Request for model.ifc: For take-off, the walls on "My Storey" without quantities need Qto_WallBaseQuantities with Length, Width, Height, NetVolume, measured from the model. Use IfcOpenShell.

First a look at what the model holds.

```python
import ifcopenshell
import ifcopenshell.util.element
import ifcopenshell.util.unit

model = ifcopenshell.open("model.ifc")
print(model.schema)
for unit_type in ("LENGTHUNIT", "AREAUNIT", "VOLUMEUNIT"):
    print(unit_type, ifcopenshell.util.unit.calculate_unit_scale(model, unit_type))
storey = next(s for s in model.by_type("IfcBuildingStorey") if s.Name == "My Storey")
walls = [e for e in ifcopenshell.util.element.get_decomposition(storey) if e.is_a("IfcWall")]
for e in sorted(walls, key=lambda e: e.id()):
    print(e.id(), e.is_a(), e.Name, list(ifcopenshell.util.element.get_psets(e, qtos_only=True)), sep=" | ")
```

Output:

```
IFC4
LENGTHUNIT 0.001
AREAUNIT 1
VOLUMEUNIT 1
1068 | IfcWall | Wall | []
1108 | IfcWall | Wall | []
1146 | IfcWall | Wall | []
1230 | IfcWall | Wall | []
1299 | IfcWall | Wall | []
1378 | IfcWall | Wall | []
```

```python
import ifcopenshell
import ifcopenshell.api.pset
import ifcopenshell.geom
import ifcopenshell.util.element
import ifcopenshell.util.shape
import ifcopenshell.util.unit

model = ifcopenshell.open("model.ifc")
unit_scale = ifcopenshell.util.unit.calculate_unit_scale(model)
volume_scale = ifcopenshell.util.unit.calculate_unit_scale(model, "VOLUMEUNIT")
settings = ifcopenshell.geom.settings()

storey = next(s for s in model.by_type("IfcBuildingStorey") if s.Name == "My Storey")
walls = [e for e in ifcopenshell.util.element.get_decomposition(storey) if e.is_a("IfcWall")]

for e in sorted(walls, key=lambda e: e.id()):
    if ifcopenshell.util.element.get_psets(e, qtos_only=True, should_inherit=False):
        continue
    # Geometry comes back in metres, in the element's own axes.
    shape = ifcopenshell.geom.create_shape(settings, e)
    values = {
        "Length": ifcopenshell.util.shape.get_x(shape.geometry) / unit_scale,
        "Width": ifcopenshell.util.shape.get_y(shape.geometry) / unit_scale,
        "Height": ifcopenshell.util.shape.get_z(shape.geometry) / unit_scale,
        "NetVolume": ifcopenshell.util.shape.get_volume(shape.geometry) / volume_scale,
    }
    qto = ifcopenshell.api.pset.add_qto(model, product=e, name="Qto_WallBaseQuantities")
    ifcopenshell.api.pset.edit_qto(model, qto=qto, properties=values)
    print(e.id(), {k: round(v, 3) for k, v in values.items()})

model.write("model_v2.ifc")
```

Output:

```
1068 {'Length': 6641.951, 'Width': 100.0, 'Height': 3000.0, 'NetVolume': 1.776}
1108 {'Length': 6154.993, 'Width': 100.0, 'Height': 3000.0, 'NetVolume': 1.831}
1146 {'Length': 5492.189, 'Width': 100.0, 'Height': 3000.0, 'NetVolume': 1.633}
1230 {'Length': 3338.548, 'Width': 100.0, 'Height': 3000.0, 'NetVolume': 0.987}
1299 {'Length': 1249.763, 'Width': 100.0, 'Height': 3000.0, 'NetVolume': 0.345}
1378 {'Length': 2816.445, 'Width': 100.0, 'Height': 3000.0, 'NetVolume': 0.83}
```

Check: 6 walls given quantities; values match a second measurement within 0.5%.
